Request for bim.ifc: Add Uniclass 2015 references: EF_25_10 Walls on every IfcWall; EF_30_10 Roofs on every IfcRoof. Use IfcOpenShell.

First a look at what the model holds.

```python
import ifcopenshell

model = ifcopenshell.open("bim.ifc")
print(model.schema)
print("classifications:", [c.Name for c in model.by_type("IfcClassification")])
for ifc_class in ("IfcDoor", "IfcRoof", "IfcStair", "IfcWall", "IfcWindow"):
    print(ifc_class, len(model.by_type(ifc_class)))
```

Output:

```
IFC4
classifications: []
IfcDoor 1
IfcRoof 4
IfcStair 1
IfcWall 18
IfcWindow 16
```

```python
import ifcopenshell
import ifcopenshell.api.classification

model = ifcopenshell.open("bim.ifc")

system = ifcopenshell.api.classification.add_classification(model, classification="Uniclass 2015")

codes = {
    "IfcWall": ("EF_25_10", "Walls"),
    "IfcRoof": ("EF_30_10", "Roofs"),
}
for ifc_class, (code, name) in codes.items():
    products = model.by_type(ifc_class)
    ifcopenshell.api.classification.add_reference(
        model, products=products, classification=system, identification=code, name=name
    )
    print(code, len(products))

model.write("bim-out.ifc")
```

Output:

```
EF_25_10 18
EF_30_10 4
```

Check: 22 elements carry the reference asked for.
